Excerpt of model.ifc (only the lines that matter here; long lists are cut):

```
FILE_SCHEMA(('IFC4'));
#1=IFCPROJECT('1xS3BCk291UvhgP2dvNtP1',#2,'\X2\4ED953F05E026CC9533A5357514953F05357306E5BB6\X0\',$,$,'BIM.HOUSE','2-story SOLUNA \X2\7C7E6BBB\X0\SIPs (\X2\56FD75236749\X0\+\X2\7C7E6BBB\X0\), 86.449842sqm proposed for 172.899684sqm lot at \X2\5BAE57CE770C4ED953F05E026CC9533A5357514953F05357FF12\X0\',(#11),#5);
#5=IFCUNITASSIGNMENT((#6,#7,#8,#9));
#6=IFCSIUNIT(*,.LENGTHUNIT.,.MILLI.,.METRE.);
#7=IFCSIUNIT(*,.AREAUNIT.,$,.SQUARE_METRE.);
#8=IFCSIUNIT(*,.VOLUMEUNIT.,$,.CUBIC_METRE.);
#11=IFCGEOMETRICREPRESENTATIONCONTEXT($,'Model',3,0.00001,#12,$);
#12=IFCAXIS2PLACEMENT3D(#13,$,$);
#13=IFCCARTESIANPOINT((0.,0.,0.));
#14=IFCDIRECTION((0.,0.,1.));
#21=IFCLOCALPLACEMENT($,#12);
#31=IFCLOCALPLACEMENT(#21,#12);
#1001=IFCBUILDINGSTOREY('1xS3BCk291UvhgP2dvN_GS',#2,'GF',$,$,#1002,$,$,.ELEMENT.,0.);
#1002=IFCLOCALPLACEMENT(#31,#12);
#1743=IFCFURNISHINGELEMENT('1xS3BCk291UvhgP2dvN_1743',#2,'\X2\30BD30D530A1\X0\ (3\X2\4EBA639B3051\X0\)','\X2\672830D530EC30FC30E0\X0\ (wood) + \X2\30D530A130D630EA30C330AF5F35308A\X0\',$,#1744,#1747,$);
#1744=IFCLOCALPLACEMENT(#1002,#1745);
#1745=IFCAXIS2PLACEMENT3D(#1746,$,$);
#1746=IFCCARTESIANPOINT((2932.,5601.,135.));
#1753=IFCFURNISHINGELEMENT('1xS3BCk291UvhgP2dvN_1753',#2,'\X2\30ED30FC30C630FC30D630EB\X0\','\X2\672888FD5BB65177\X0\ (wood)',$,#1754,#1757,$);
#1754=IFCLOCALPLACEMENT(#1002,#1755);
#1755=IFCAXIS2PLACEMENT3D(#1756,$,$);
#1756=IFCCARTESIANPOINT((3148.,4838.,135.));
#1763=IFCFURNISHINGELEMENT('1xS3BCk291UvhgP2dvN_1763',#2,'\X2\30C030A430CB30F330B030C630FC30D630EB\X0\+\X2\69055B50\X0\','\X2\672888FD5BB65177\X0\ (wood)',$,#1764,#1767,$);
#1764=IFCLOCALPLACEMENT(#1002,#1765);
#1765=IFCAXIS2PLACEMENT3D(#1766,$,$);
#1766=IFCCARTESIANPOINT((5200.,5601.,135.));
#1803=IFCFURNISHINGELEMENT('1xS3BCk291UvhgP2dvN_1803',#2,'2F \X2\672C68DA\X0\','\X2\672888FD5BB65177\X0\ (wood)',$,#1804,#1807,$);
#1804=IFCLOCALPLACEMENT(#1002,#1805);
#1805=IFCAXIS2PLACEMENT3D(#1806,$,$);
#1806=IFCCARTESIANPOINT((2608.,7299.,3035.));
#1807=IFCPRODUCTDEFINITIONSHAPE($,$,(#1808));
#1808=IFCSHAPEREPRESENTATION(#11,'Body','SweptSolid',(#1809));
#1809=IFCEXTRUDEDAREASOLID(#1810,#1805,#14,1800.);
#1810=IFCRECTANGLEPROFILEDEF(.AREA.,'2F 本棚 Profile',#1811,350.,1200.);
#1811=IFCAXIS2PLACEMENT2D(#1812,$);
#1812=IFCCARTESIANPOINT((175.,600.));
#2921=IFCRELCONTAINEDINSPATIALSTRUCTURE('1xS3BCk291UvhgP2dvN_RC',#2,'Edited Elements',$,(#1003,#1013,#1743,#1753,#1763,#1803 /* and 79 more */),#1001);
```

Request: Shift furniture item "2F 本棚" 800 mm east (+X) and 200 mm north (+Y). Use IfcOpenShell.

```python
import ifcopenshell
import ifcopenshell.api.geometry
import ifcopenshell.util.placement
import ifcopenshell.util.unit

model = ifcopenshell.open("model.ifc")
unit_scale = ifcopenshell.util.unit.calculate_unit_scale(model)

item = model.by_guid("1xS3BCk291UvhgP2dvN_1803")
matrix = ifcopenshell.util.placement.get_local_placement(item.ObjectPlacement)
matrix[0, 3] += 0.8 / unit_scale
matrix[1, 3] += 0.2 / unit_scale
ifcopenshell.api.geometry.edit_object_placement(model, product=item, matrix=matrix, is_si=False)

print(ifcopenshell.util.placement.get_local_placement(item.ObjectPlacement).round(3) + 0.0)

model.write("model_edited.ifc")
```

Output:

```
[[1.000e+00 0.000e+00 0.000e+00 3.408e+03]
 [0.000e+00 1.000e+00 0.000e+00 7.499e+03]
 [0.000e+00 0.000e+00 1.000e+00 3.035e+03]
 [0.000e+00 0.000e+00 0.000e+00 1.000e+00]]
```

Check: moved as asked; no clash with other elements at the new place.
